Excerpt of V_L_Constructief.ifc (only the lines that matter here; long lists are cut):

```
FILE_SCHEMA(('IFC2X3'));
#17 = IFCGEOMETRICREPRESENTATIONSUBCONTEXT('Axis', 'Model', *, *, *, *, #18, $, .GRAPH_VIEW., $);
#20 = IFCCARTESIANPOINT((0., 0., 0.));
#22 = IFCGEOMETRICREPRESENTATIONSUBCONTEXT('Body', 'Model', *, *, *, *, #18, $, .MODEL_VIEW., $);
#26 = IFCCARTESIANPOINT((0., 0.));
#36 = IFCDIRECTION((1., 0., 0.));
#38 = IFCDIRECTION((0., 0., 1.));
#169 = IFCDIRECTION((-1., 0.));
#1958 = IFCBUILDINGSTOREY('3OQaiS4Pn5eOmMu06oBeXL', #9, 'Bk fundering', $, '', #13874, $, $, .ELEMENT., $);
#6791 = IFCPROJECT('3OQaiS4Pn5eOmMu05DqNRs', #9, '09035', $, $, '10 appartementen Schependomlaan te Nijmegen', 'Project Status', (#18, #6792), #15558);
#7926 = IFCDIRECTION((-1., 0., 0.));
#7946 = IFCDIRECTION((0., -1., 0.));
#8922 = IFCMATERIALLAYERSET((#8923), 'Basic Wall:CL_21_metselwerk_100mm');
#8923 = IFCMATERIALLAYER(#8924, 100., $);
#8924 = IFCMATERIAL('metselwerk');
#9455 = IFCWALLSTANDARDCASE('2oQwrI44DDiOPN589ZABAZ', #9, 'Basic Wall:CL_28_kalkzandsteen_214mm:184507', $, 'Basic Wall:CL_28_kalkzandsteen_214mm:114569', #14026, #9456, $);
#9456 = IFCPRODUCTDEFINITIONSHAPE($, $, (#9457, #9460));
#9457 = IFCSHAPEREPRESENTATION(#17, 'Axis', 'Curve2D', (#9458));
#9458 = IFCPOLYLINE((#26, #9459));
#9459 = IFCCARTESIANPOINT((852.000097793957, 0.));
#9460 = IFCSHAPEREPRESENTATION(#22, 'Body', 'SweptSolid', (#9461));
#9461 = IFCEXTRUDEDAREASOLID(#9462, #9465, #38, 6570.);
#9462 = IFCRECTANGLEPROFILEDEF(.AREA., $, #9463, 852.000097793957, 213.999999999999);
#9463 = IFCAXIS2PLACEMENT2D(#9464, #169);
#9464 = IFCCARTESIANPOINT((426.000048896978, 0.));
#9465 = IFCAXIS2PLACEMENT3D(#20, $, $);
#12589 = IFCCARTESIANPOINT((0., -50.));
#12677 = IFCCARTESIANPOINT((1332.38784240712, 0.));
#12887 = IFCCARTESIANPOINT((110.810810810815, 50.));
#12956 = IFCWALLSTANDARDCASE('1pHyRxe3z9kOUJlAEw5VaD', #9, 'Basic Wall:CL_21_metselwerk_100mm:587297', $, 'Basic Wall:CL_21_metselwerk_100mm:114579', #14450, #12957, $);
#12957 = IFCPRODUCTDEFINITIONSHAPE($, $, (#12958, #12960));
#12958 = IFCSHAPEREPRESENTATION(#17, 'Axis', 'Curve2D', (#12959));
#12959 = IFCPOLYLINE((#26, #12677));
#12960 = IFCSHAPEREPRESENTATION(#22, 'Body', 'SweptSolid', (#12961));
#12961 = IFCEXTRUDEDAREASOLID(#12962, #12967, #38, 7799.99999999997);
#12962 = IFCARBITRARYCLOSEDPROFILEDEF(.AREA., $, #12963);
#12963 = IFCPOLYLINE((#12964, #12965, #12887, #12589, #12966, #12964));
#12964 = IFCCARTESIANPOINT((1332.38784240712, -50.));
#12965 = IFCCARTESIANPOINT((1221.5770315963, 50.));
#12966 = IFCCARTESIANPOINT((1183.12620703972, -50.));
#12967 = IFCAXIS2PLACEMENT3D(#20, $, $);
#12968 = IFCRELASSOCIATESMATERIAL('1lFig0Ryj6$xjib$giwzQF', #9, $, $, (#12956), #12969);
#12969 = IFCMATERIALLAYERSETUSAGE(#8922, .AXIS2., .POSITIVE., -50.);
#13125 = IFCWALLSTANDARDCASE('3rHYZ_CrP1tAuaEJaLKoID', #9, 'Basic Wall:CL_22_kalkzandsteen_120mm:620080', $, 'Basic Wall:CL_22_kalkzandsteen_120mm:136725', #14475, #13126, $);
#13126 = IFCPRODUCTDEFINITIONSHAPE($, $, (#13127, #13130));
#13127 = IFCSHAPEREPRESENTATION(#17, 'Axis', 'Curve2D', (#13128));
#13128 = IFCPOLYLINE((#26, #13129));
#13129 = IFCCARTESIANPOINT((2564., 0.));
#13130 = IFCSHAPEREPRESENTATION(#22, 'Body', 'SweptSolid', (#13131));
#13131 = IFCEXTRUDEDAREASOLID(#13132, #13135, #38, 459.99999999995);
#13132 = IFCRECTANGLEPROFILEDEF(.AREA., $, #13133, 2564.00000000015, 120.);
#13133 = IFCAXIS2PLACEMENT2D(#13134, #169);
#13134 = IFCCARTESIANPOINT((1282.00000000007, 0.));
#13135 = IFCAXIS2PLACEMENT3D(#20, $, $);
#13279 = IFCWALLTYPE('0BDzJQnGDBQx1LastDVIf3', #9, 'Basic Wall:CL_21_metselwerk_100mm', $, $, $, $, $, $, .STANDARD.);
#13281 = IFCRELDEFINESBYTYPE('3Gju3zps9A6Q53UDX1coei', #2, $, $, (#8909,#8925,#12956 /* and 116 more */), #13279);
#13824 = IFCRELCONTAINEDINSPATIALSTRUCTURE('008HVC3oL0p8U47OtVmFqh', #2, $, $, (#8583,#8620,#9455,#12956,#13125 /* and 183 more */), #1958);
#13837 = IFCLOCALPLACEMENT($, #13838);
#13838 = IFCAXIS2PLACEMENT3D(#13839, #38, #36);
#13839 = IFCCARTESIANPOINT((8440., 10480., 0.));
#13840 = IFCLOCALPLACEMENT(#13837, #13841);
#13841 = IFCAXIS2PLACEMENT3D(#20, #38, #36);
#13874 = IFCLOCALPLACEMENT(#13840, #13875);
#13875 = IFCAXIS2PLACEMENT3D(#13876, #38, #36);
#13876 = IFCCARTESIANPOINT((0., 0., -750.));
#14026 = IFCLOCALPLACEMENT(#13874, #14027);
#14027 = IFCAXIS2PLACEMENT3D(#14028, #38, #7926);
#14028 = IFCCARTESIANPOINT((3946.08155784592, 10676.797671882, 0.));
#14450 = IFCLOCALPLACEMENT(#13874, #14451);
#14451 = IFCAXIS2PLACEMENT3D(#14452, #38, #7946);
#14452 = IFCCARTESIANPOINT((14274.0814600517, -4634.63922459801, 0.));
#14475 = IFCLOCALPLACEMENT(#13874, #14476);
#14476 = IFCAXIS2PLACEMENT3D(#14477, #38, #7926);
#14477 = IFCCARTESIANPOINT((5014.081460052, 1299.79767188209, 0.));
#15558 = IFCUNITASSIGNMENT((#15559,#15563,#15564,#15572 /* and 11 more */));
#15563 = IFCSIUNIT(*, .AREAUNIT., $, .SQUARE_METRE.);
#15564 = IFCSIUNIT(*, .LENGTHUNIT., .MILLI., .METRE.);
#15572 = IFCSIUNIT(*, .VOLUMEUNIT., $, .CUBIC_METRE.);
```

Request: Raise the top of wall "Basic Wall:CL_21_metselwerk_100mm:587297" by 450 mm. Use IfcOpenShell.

```python
import ifcopenshell
import ifcopenshell.geom
import ifcopenshell.util.representation
import ifcopenshell.util.shape
import ifcopenshell.util.unit

model = ifcopenshell.open("V_L_Constructief.ifc")
unit_scale = ifcopenshell.util.unit.calculate_unit_scale(model)
settings = ifcopenshell.geom.settings()


def volume(element):
    """Net volume in cubic metres, openings subtracted."""
    shape = ifcopenshell.geom.create_shape(settings, element)
    return ifcopenshell.util.shape.get_volume(shape.geometry)


wall = model.by_guid("1pHyRxe3z9kOUJlAEw5VaD")
before = volume(wall)

body = ifcopenshell.util.representation.get_representation(wall, "Model", "Body")
solid = body.Items[0]
old_height = solid.Depth
solid.Depth += 0.45 / unit_scale
after = volume(wall)

print(f"height {old_height:g} -> {solid.Depth:g}, volume {before:.3f} -> {after:.3f} m3")

model.write("V_L_Constructief_rev.ifc")
```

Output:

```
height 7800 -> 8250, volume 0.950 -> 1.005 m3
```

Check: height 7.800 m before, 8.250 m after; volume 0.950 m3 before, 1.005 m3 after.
